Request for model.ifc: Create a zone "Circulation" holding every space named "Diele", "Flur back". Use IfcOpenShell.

First a look at what the model holds.

```python
import ifcopenshell

model = ifcopenshell.open("model.ifc")
print(model.schema)
seen = {}
for space in model.by_type("IfcSpace"):
    seen[space.LongName] = seen.get(space.LongName, 0) + 1
for name, count in sorted(seen.items(), key=str):
    print(count, "x", name)
print("zones:", [z.Name for z in model.by_type("IfcZone")][:20])
```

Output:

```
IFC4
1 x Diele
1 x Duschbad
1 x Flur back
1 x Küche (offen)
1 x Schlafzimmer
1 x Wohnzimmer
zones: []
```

```python
import ifcopenshell
import ifcopenshell.api.group
import ifcopenshell.api.root

model = ifcopenshell.open("model.ifc")

names = {"Diele", "Flur back"}
spaces = [s for s in model.by_type("IfcSpace") if s.LongName in names]

zone = ifcopenshell.api.root.create_entity(model, ifc_class="IfcZone", name="Circulation")
ifcopenshell.api.group.assign_group(model, products=spaces, group=zone)
print(len(spaces), "spaces in", zone.Name)

model.write("model_edited.ifc")
```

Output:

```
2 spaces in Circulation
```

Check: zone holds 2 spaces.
